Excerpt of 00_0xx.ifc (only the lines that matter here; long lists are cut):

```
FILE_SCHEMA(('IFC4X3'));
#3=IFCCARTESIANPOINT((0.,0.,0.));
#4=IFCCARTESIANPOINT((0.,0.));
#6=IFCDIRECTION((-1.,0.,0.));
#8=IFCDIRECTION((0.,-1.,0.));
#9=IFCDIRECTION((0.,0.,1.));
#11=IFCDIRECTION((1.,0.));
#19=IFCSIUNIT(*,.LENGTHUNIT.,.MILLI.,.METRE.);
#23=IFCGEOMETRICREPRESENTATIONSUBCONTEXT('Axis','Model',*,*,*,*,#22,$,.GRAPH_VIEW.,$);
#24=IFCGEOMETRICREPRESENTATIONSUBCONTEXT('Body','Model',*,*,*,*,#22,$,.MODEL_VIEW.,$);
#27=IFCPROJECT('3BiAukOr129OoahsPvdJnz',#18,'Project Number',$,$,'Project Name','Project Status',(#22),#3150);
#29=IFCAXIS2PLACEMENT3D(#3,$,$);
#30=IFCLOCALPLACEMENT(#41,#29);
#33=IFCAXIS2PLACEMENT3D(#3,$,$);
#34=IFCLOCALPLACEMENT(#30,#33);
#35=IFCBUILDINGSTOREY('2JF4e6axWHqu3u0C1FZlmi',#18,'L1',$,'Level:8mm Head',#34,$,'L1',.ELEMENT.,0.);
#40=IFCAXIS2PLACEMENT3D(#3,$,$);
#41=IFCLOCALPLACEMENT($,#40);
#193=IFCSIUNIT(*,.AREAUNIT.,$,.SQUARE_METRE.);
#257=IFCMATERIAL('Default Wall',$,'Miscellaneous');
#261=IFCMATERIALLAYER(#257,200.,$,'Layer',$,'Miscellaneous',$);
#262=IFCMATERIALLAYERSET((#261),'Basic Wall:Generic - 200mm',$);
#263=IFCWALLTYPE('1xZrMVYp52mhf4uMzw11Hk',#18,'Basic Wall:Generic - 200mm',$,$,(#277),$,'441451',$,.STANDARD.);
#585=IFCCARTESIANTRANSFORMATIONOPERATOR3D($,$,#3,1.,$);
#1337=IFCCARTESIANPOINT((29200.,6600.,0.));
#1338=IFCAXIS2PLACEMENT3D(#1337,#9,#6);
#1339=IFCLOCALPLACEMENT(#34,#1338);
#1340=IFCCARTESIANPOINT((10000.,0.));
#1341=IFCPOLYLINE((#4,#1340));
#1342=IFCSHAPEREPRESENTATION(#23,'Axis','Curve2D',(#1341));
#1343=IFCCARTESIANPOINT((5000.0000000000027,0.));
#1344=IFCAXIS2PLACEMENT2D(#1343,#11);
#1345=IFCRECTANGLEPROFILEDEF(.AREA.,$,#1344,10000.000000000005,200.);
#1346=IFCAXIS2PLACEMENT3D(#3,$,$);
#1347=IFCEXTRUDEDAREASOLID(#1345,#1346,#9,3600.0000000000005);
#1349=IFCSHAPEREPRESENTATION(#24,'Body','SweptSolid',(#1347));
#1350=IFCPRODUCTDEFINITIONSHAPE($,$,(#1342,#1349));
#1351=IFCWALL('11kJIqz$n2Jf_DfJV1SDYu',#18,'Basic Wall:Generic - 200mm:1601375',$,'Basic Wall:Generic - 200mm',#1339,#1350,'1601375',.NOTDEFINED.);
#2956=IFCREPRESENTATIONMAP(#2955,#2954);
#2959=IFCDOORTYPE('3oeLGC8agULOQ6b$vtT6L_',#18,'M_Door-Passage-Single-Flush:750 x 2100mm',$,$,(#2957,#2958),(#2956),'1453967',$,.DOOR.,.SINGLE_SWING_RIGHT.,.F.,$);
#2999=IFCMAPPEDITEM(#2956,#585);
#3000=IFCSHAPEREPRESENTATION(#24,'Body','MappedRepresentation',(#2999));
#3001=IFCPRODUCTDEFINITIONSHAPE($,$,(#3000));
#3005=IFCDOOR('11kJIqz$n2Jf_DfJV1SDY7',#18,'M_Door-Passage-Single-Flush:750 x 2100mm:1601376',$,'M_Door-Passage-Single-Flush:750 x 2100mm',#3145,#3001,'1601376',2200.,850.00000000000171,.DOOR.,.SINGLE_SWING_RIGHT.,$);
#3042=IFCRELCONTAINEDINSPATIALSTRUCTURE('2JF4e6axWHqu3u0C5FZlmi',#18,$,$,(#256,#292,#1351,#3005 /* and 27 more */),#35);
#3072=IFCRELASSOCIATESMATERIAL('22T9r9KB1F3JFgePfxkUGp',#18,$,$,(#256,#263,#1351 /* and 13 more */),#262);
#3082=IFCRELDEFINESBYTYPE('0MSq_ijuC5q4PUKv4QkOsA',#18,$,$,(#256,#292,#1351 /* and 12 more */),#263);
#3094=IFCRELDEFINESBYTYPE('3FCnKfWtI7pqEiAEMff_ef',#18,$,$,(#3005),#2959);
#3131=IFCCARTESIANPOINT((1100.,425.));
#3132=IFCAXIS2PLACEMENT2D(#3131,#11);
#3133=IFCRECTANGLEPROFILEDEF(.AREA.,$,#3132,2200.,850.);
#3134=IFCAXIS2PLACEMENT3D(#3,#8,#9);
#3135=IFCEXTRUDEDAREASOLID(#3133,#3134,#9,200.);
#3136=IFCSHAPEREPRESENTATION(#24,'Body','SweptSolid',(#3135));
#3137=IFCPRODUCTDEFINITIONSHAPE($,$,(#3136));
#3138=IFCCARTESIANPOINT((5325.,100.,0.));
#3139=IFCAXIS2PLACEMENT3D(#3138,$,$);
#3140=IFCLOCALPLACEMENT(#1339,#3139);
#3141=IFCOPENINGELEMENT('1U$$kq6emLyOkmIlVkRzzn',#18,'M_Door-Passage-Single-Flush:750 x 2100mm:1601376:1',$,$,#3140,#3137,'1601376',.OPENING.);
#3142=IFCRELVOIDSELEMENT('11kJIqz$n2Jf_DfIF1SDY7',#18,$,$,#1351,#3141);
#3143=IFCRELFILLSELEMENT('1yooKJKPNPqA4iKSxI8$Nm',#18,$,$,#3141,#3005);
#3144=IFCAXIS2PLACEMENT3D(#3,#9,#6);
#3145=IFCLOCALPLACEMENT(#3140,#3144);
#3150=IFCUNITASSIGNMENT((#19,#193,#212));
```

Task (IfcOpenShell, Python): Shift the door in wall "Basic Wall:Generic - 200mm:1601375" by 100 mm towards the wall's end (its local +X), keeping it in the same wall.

```python
import ifcopenshell
import ifcopenshell.api.geometry
import ifcopenshell.util.placement

model = ifcopenshell.open("00_0xx.ifc")

door = model.by_guid("11kJIqz$n2Jf_DfJV1SDY7")
opening = door.FillsVoids[0].RelatingOpeningElement
wall = opening.VoidsElements[0].RelatingBuildingElement

wall_matrix = ifcopenshell.util.placement.get_local_placement(wall.ObjectPlacement)
shift = wall_matrix[:3, 0] * 100.0
before = ifcopenshell.util.placement.get_local_placement(door.ObjectPlacement)[:3, 3].copy()

# The door is placed relative to its opening, so it follows when the opening moves.
matrix = ifcopenshell.util.placement.get_local_placement(opening.ObjectPlacement)
matrix[:3, 3] += shift
ifcopenshell.api.geometry.edit_object_placement(
    model, product=opening, matrix=matrix, is_si=False, should_transform_children=True
)

after = ifcopenshell.util.placement.get_local_placement(door.ObjectPlacement)[:3, 3]
print("door moved by", (after - before).round(3) + 0.0)

model.write("00_0xx_rev.ifc")
```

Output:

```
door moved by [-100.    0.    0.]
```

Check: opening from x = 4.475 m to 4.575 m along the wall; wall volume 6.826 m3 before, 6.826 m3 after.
